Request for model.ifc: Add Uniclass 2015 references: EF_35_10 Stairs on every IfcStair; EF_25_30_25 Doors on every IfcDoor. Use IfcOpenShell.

First a look at what the model holds.

```python
import ifcopenshell

model = ifcopenshell.open("model.ifc")
print(model.schema)
print("classifications:", [c.Name for c in model.by_type("IfcClassification")])
for ifc_class in ("IfcDoor", "IfcRoof", "IfcStair", "IfcWall", "IfcWindow"):
    print(ifc_class, len(model.by_type(ifc_class)))
```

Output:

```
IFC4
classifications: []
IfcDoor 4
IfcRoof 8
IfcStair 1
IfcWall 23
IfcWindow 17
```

```python
import ifcopenshell
import ifcopenshell.api.classification

model = ifcopenshell.open("model.ifc")

system = ifcopenshell.api.classification.add_classification(model, classification="Uniclass 2015")

codes = {
    "IfcStair": ("EF_35_10", "Stairs"),
    "IfcDoor": ("EF_25_30_25", "Doors"),
}
for ifc_class, (code, name) in codes.items():
    products = model.by_type(ifc_class)
    ifcopenshell.api.classification.add_reference(
        model, products=products, classification=system, identification=code, name=name
    )
    print(code, len(products))

model.write("model_edited.ifc")
```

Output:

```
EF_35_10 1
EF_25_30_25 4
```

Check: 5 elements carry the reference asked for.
